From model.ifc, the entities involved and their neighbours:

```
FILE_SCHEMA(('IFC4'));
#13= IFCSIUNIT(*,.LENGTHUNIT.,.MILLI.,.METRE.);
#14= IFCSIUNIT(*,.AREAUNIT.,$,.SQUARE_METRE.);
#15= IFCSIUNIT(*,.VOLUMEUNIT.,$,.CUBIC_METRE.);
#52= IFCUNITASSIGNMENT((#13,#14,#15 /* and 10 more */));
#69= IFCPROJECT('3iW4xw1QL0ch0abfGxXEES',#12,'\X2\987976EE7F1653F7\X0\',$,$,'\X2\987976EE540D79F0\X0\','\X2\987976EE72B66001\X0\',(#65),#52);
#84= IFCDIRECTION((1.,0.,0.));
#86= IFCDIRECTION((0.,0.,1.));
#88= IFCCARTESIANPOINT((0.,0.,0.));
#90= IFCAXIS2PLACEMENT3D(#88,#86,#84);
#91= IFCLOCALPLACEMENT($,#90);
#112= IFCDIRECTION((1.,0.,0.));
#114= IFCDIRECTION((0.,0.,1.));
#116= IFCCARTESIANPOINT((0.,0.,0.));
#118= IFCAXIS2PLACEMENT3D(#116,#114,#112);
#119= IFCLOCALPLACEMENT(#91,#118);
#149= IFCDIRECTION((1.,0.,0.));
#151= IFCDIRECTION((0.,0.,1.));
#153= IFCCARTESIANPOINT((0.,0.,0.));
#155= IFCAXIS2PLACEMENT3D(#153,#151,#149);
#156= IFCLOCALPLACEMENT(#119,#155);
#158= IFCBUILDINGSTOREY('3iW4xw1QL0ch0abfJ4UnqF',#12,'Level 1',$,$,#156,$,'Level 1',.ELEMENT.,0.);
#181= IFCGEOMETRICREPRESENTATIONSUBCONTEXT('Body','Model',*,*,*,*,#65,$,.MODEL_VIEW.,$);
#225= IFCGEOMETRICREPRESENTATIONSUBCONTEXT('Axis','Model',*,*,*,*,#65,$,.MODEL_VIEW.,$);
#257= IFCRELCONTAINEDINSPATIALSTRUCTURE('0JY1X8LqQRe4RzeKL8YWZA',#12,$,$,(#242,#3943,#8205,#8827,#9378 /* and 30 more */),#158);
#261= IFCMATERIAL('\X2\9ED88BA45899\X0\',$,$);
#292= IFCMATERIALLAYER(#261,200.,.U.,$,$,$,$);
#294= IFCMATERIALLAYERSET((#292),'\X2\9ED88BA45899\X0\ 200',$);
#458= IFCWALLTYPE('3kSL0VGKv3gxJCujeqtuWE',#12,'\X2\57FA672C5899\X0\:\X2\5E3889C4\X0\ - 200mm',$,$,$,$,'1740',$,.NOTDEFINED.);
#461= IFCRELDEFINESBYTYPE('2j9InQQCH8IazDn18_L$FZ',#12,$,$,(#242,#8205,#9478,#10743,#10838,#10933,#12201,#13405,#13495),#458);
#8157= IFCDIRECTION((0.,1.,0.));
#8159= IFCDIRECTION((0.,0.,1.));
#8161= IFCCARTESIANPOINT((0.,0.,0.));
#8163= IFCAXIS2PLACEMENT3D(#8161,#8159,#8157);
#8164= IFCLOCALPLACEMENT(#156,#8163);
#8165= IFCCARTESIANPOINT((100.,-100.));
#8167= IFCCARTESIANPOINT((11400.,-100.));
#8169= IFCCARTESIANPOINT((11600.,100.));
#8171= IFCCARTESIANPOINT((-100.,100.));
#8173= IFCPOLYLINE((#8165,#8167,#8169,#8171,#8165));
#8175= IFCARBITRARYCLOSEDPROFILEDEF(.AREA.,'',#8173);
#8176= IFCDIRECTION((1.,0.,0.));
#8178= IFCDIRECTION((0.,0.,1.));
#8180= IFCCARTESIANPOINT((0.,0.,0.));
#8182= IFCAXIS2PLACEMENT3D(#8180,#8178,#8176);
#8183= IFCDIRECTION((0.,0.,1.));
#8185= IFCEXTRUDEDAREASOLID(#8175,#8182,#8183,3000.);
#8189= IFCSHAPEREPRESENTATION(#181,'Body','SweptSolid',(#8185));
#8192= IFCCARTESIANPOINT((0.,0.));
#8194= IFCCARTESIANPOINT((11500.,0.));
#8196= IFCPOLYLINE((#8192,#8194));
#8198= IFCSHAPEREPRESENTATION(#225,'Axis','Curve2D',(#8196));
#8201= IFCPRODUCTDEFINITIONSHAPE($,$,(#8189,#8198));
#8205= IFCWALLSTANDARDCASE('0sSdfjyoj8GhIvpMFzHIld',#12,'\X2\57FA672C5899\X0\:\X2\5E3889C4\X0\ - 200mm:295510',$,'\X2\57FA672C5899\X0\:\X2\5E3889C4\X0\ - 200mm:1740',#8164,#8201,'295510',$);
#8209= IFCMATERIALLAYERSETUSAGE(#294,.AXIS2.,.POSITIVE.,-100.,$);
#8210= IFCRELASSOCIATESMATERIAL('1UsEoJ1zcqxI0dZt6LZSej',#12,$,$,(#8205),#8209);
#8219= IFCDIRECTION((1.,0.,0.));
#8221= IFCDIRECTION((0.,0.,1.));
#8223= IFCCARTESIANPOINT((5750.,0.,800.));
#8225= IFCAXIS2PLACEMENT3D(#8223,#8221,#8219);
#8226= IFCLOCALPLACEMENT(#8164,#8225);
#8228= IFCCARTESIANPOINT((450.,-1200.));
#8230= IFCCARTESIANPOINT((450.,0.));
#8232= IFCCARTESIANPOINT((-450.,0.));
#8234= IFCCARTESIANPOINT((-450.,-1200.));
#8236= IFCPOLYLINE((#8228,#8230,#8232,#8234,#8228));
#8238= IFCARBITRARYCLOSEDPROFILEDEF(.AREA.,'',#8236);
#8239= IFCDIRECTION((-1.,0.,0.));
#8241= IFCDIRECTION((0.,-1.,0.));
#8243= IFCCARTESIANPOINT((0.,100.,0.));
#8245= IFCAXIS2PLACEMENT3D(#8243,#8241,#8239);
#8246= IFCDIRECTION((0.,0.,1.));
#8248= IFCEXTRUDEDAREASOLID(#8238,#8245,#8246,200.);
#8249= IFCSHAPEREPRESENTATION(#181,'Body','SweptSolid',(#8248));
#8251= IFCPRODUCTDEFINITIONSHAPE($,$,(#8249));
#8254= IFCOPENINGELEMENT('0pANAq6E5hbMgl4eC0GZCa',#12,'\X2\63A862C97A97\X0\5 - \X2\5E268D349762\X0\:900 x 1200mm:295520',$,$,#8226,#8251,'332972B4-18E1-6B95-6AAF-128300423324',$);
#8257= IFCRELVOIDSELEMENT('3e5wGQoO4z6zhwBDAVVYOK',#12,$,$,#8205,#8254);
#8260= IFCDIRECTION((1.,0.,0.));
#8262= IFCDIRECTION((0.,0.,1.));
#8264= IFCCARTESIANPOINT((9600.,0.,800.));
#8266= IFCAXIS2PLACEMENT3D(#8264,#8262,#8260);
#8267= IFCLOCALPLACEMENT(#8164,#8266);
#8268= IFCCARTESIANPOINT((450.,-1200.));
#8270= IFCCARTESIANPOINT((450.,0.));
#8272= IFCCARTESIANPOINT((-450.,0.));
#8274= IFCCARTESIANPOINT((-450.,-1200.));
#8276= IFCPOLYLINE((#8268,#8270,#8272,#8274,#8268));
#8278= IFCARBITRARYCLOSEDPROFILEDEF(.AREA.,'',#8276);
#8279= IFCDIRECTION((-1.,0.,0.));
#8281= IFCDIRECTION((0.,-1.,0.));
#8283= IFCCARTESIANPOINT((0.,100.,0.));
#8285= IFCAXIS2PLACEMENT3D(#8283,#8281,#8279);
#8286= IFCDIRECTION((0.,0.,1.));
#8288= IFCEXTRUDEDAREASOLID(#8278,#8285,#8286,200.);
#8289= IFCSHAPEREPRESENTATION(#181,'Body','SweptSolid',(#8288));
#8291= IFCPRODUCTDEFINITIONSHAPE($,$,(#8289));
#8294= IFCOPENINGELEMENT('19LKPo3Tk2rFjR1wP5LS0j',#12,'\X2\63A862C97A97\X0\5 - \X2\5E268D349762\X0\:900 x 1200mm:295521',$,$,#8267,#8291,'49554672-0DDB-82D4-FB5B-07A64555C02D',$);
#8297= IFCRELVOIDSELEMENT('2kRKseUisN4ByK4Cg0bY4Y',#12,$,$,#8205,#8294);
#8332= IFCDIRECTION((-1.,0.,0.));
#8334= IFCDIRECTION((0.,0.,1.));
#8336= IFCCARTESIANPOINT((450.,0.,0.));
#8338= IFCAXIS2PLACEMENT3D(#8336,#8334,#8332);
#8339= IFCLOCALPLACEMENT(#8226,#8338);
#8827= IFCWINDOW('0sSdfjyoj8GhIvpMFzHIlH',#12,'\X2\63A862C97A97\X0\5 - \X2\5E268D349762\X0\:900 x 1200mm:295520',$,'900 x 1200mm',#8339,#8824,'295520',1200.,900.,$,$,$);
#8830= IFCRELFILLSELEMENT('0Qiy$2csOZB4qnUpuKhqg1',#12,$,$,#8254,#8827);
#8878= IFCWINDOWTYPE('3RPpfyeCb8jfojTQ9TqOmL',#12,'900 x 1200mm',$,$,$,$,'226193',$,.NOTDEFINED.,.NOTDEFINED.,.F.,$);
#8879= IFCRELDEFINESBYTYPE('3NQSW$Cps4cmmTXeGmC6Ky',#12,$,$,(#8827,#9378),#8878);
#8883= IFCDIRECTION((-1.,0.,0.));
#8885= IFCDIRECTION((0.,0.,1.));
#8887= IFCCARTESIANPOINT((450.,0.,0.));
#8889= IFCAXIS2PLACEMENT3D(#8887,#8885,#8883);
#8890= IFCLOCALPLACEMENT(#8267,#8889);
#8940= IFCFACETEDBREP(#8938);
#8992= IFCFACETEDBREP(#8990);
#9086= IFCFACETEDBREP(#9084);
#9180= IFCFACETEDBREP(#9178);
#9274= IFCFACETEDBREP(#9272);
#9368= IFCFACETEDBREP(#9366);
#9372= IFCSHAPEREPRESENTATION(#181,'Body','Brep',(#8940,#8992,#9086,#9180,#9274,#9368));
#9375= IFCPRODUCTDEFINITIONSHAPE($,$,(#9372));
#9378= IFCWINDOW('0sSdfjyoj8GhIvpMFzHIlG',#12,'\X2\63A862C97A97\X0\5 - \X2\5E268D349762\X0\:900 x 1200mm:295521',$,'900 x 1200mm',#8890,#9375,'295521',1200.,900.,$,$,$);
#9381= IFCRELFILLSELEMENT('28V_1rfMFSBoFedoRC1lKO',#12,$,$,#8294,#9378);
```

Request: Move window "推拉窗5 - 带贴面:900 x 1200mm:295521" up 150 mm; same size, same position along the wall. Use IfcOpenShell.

```python
import numpy as np
import ifcopenshell
import ifcopenshell.api.geometry
import ifcopenshell.util.placement
import ifcopenshell.util.unit

model = ifcopenshell.open("model.ifc")
unit_scale = ifcopenshell.util.unit.calculate_unit_scale(model)

window = model.by_id(9378)
opening = window.FillsVoids[0].RelatingOpeningElement
dz = 150.0

shift = np.array([0.0, 0.0, dz])
# The window is placed relative to its opening, so it follows when the opening moves.
matrix = ifcopenshell.util.placement.get_local_placement(opening.ObjectPlacement)
matrix[:3, 3] += shift
ifcopenshell.api.geometry.edit_object_placement(
    model, product=opening, matrix=matrix, is_si=False, should_transform_children=True
)

print(f"moved by {dz * unit_scale:+.3f} m")

model.write("model-out.ifc")
```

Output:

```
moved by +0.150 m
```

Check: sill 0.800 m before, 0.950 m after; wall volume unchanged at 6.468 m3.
